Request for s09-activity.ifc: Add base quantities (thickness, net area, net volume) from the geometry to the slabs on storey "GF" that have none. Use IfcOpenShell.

First a look at what the model holds.

```python
import ifcopenshell
import ifcopenshell.util.element
import ifcopenshell.util.unit

model = ifcopenshell.open("s09-activity.ifc")
print(model.schema)
for unit_type in ("LENGTHUNIT", "AREAUNIT", "VOLUMEUNIT"):
    print(unit_type, ifcopenshell.util.unit.calculate_unit_scale(model, unit_type))
storey = next(s for s in model.by_type("IfcBuildingStorey") if s.Name == "GF")
slabs = [e for e in ifcopenshell.util.element.get_decomposition(storey) if e.is_a("IfcSlab")]
for e in sorted(slabs, key=lambda e: e.id()):
    print(e.id(), e.is_a(), e.Name, list(ifcopenshell.util.element.get_psets(e, qtos_only=True)), sep=" | ")
```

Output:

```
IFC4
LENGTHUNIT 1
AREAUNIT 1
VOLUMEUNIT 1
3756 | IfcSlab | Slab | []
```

```python
import ifcopenshell
import ifcopenshell.api.pset
import ifcopenshell.geom
import ifcopenshell.util.element
import ifcopenshell.util.shape
import ifcopenshell.util.unit

model = ifcopenshell.open("s09-activity.ifc")
unit_scale = ifcopenshell.util.unit.calculate_unit_scale(model)
area_scale = ifcopenshell.util.unit.calculate_unit_scale(model, "AREAUNIT")
volume_scale = ifcopenshell.util.unit.calculate_unit_scale(model, "VOLUMEUNIT")
settings = ifcopenshell.geom.settings()

storey = next(s for s in model.by_type("IfcBuildingStorey") if s.Name == "GF")
slabs = [e for e in ifcopenshell.util.element.get_decomposition(storey) if e.is_a("IfcSlab")]

for e in sorted(slabs, key=lambda e: e.id()):
    if ifcopenshell.util.element.get_psets(e, qtos_only=True, should_inherit=False):
        continue
    # Geometry comes back in metres, in the element's own axes.
    shape = ifcopenshell.geom.create_shape(settings, e)
    values = {
        "Width": ifcopenshell.util.shape.get_z(shape.geometry) / unit_scale,
        "NetArea": ifcopenshell.util.shape.get_footprint_area(shape.geometry) / area_scale,
        "NetVolume": ifcopenshell.util.shape.get_volume(shape.geometry) / volume_scale,
    }
    qto = ifcopenshell.api.pset.add_qto(model, product=e, name="Qto_SlabBaseQuantities")
    ifcopenshell.api.pset.edit_qto(model, qto=qto, properties=values)
    print(e.id(), {k: round(v, 3) for k, v in values.items()})

model.write("s09-activity_v2.ifc")
```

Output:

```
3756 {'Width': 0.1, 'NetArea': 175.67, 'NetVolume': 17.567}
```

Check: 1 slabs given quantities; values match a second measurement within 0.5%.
